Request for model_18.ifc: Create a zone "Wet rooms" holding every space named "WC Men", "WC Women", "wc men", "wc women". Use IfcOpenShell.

First a look at what the model holds.

```python
import ifcopenshell

model = ifcopenshell.open("model_18.ifc")
print(model.schema)
seen = {}
for space in model.by_type("IfcSpace"):
    seen[space.LongName] = seen.get(space.LongName, 0) + 1
for name, count in sorted(seen.items(), key=str):
    print(count, "x", name)
print("zones:", [z.Name for z in model.by_type("IfcZone")][:20])
```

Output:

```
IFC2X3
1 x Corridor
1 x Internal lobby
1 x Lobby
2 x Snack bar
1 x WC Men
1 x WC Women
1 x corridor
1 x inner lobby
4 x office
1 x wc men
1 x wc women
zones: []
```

```python
import ifcopenshell
import ifcopenshell.api.group
import ifcopenshell.api.root

model = ifcopenshell.open("model_18.ifc")

names = {"WC Men", "WC Women", "wc men", "wc women"}
spaces = [s for s in model.by_type("IfcSpace") if s.LongName in names]

zone = ifcopenshell.api.root.create_entity(model, ifc_class="IfcZone", name="Wet rooms")
ifcopenshell.api.group.assign_group(model, products=spaces, group=zone)
print(len(spaces), "spaces in", zone.Name)

model.write("model_18_updated.ifc")
```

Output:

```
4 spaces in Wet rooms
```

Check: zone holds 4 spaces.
